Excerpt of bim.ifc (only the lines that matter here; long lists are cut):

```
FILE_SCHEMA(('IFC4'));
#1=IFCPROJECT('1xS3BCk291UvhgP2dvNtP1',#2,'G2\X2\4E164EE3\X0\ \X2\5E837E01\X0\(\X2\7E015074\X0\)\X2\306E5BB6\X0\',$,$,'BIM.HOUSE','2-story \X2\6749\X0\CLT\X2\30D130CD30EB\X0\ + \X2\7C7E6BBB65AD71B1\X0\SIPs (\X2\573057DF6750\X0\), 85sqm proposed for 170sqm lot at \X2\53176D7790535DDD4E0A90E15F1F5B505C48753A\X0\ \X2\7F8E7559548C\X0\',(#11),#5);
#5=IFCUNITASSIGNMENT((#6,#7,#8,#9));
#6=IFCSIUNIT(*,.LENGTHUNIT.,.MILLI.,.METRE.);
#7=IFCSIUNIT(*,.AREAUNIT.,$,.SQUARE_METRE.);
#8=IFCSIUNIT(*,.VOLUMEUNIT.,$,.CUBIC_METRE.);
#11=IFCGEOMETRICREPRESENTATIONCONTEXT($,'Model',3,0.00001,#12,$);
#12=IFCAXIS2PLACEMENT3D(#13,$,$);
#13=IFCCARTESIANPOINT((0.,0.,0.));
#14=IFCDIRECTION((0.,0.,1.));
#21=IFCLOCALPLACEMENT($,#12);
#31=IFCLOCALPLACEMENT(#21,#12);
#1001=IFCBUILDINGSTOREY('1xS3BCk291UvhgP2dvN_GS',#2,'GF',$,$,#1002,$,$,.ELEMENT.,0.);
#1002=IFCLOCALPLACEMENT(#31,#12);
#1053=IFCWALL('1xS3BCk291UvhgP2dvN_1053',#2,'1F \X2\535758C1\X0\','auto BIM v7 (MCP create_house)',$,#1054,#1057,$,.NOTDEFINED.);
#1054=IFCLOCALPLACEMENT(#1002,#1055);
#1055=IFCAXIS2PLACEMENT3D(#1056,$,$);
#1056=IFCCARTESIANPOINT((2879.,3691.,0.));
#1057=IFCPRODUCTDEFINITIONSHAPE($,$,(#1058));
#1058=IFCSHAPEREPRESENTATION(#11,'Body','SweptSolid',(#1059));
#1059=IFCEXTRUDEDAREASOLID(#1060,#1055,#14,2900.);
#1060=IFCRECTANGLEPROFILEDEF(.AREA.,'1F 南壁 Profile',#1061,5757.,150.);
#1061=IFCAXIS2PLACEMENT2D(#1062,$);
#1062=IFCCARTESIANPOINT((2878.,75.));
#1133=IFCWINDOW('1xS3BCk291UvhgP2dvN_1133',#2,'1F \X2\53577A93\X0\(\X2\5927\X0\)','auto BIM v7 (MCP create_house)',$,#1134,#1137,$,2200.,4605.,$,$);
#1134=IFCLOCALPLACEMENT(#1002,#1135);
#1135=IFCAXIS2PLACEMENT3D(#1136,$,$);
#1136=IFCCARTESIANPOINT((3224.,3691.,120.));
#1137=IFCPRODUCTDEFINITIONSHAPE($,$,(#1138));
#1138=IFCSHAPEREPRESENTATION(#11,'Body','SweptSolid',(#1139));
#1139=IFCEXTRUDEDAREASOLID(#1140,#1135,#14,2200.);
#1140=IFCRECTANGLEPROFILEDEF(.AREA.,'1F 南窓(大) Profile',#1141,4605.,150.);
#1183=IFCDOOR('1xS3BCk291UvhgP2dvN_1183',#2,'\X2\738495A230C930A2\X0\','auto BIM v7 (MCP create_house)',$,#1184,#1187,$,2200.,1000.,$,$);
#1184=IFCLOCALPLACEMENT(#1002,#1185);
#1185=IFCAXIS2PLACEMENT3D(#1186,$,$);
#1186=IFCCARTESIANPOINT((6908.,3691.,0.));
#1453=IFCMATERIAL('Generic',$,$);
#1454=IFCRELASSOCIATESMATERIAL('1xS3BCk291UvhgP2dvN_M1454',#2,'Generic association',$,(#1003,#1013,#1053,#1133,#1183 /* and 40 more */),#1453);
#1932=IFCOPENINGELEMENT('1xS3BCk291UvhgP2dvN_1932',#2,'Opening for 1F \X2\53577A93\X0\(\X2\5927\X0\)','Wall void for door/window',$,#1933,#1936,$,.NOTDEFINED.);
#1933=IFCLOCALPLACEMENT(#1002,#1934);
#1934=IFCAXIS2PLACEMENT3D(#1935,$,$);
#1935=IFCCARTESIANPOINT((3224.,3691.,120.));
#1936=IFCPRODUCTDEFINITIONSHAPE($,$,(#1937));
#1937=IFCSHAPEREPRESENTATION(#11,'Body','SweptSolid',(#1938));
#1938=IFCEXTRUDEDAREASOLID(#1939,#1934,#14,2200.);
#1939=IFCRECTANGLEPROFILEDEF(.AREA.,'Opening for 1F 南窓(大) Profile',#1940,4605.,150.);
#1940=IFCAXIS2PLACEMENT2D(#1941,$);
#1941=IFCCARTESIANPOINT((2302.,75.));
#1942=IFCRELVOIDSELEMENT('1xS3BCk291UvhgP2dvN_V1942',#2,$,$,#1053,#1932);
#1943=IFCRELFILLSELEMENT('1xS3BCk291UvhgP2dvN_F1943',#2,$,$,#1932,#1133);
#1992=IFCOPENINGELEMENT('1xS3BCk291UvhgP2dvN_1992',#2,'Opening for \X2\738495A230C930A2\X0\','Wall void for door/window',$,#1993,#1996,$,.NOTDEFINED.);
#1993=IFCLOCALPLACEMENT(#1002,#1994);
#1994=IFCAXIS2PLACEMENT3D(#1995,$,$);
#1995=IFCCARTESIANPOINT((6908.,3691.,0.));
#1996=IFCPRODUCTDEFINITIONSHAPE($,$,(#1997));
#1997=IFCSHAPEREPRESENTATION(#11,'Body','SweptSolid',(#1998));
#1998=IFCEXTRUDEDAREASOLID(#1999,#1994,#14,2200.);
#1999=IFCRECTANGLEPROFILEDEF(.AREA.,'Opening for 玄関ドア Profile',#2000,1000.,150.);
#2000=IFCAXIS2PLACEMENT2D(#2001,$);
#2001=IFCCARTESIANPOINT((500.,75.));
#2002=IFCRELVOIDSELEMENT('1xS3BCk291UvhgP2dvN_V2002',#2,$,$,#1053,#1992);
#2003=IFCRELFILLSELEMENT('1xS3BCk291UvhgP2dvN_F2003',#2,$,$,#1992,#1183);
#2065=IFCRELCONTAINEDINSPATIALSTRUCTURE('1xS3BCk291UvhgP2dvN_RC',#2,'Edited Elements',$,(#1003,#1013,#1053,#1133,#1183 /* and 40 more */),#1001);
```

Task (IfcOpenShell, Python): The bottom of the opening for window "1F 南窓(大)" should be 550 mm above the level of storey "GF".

```python
import numpy as np
import ifcopenshell
import ifcopenshell.api.geometry
import ifcopenshell.geom
import ifcopenshell.util.element
import ifcopenshell.util.placement
import ifcopenshell.util.shape
import ifcopenshell.util.unit

model = ifcopenshell.open("bim.ifc")
unit_scale = ifcopenshell.util.unit.calculate_unit_scale(model)

window = model.by_id(1133)
opening = window.FillsVoids[0].RelatingOpeningElement
storey = ifcopenshell.util.element.get_container(window, ifc_class="IfcBuildingStorey")
level = ifcopenshell.util.placement.get_local_placement(storey.ObjectPlacement)[2, 3]

# The opening's origin need not be at the sill, so measure its lowest point.
shape = ifcopenshell.geom.create_shape(ifcopenshell.geom.settings(), opening)
bottom = ifcopenshell.util.shape.get_shape_bottom_elevation(shape, shape.geometry) / unit_scale
dz = level + 550.0 - bottom

shift = np.array([0.0, 0.0, dz])
# The window is not placed relative to its opening, so move both.
for product in (opening, window):
    matrix = ifcopenshell.util.placement.get_local_placement(product.ObjectPlacement)
    matrix[:3, 3] += shift
    ifcopenshell.api.geometry.edit_object_placement(model, product=product, matrix=matrix, is_si=False)

print(f"moved by {dz * unit_scale:+.3f} m")

model.write("bim_rev.ifc")
```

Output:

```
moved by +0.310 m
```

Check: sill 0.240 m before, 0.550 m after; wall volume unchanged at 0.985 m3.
